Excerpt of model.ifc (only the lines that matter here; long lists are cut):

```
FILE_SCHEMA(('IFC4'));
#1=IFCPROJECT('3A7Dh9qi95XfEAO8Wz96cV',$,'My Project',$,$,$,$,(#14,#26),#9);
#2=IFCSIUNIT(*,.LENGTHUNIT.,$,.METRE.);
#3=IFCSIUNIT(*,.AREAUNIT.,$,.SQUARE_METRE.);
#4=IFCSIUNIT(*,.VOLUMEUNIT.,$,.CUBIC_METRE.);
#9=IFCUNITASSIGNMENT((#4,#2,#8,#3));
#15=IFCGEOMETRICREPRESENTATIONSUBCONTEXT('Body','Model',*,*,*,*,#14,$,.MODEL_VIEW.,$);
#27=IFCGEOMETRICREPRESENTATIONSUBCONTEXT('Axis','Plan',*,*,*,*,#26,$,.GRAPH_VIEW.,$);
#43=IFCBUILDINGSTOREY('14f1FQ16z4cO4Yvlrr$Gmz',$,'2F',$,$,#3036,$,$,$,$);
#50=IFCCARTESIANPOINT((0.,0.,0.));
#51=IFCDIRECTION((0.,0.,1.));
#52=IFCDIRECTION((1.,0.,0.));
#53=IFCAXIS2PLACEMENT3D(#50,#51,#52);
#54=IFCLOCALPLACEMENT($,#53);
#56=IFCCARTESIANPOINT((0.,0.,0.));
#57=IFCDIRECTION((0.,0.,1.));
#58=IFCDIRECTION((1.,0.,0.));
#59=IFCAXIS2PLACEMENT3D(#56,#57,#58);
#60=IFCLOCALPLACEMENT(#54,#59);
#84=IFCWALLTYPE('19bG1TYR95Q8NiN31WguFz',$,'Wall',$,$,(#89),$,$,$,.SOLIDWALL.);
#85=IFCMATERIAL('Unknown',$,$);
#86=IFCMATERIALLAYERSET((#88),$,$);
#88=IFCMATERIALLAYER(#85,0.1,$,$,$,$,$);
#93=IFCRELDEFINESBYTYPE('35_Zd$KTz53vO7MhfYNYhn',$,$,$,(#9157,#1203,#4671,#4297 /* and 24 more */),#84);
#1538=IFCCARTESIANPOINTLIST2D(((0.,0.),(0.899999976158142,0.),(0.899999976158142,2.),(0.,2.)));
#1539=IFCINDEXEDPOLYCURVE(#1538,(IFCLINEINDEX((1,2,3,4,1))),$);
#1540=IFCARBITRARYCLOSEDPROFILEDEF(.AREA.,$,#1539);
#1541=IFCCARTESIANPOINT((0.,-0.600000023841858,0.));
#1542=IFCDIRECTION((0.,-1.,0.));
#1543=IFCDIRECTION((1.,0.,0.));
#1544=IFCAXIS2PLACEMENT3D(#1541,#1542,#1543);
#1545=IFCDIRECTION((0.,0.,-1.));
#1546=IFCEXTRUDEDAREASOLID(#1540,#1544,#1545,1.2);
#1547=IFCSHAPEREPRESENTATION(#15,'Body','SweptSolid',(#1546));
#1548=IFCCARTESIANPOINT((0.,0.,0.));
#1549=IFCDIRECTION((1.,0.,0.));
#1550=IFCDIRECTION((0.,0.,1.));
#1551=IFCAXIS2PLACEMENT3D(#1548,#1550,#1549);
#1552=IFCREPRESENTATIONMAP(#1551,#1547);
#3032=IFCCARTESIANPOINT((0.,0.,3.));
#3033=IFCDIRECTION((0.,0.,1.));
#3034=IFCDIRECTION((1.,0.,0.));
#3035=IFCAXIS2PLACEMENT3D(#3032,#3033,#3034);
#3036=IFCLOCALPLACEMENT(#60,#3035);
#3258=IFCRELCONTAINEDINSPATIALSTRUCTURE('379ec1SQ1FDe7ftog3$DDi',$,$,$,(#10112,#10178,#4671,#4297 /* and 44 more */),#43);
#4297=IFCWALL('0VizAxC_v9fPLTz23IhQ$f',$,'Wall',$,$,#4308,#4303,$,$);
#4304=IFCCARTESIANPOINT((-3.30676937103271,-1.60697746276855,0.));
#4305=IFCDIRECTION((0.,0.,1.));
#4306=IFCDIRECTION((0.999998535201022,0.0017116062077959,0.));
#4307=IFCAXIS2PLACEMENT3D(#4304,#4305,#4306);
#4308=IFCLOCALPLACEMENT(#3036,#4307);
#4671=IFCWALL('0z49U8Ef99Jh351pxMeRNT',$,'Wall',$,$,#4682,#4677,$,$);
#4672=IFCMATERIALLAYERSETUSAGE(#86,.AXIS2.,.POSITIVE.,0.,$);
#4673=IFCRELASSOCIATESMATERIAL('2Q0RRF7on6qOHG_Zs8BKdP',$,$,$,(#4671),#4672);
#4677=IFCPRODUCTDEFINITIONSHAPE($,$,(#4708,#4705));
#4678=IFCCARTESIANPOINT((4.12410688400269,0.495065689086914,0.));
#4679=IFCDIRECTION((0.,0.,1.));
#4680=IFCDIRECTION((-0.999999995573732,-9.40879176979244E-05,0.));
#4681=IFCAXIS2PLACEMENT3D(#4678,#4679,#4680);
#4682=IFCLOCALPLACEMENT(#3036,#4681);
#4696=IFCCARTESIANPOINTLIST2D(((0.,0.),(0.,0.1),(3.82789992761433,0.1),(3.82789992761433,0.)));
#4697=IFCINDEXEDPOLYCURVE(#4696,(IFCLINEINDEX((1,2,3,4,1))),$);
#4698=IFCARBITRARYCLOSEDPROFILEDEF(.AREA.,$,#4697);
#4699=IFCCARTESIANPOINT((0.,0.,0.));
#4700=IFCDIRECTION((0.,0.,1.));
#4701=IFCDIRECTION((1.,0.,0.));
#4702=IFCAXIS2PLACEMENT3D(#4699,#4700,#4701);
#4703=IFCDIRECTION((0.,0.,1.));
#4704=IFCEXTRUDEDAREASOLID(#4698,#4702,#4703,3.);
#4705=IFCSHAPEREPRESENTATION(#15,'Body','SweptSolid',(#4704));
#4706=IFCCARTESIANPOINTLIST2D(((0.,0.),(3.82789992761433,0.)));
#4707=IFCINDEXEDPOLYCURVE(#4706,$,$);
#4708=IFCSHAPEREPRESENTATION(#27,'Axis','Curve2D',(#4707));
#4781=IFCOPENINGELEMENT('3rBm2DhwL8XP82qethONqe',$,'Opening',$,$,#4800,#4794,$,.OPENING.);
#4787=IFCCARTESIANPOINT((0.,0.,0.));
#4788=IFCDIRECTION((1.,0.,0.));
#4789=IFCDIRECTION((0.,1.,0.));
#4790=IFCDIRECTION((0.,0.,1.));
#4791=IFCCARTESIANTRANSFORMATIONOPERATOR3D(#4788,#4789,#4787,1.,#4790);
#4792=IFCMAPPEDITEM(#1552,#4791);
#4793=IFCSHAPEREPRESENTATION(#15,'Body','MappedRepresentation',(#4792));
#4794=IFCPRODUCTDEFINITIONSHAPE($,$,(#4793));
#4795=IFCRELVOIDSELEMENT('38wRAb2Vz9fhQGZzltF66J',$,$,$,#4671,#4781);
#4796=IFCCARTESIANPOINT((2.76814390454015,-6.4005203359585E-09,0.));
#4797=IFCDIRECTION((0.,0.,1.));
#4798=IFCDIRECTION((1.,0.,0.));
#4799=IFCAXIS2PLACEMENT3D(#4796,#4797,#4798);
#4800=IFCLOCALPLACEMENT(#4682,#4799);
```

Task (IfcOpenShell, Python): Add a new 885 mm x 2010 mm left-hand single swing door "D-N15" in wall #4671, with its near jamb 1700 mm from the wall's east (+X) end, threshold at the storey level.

```python
import numpy as np
import ifcopenshell
import ifcopenshell.api.feature
import ifcopenshell.api.geometry
import ifcopenshell.api.root
import ifcopenshell.api.spatial
import ifcopenshell.geom
import ifcopenshell.util.element
import ifcopenshell.util.placement
import ifcopenshell.util.representation
import ifcopenshell.util.shape
import ifcopenshell.util.unit

model = ifcopenshell.open("model.ifc")
unit_scale = ifcopenshell.util.unit.calculate_unit_scale(model)
settings = ifcopenshell.geom.settings()


def volume(element):
    """Net volume in cubic metres, openings subtracted."""
    shape = ifcopenshell.geom.create_shape(settings, element)
    return ifcopenshell.util.shape.get_volume(shape.geometry)


wall = model.by_id(4671)
storey = ifcopenshell.util.element.get_container(wall, ifc_class="IfcBuildingStorey")
context = ifcopenshell.util.representation.get_context(model, "Model", "Body", "MODEL_VIEW")
before = volume(wall)

width, height, from_end, sill = 0.885, 2.01, 1.7, 0.0  # metres

# The wall runs along its own X axis, and the end named is its -X end.
wall_shape = ifcopenshell.geom.create_shape(settings, wall)
x, y, z = ifcopenshell.util.shape.get_vertices(wall_shape.geometry).T
start = x.min() + from_end
face, thickness = float(y.min()), float(y.max() - y.min())
wall_matrix = ifcopenshell.util.placement.get_local_placement(wall.ObjectPlacement)
level = ifcopenshell.util.placement.get_local_placement(storey.ObjectPlacement)[2, 3]


def in_wall(x, y):
    """Placement at x, y metres in the wall's axes, at sill height."""
    matrix = wall_matrix.copy()
    matrix[:, 3] = wall_matrix @ np.array([x / unit_scale, y / unit_scale, 0.0, 1.0])
    matrix[2, 3] = level + sill / unit_scale
    return matrix


# Opening: a box that overshoots both wall faces by 50 mm.
opening = ifcopenshell.api.root.create_entity(model, ifc_class="IfcOpeningElement", predefined_type="OPENING")
box = ifcopenshell.api.geometry.add_wall_representation(
    model, context=context, length=width, height=height, thickness=thickness + 0.1
)
ifcopenshell.api.geometry.assign_representation(model, product=opening, representation=box)
ifcopenshell.api.geometry.edit_object_placement(model, product=opening, matrix=in_wall(start, face - 0.05), is_si=False)
ifcopenshell.api.feature.add_feature(model, feature=opening, element=wall)

door = ifcopenshell.api.root.create_entity(model, ifc_class="IfcDoor", name="D-N15", predefined_type="DOOR")
door.OverallWidth, door.OverallHeight = width / unit_scale, height / unit_scale
door.OperationType = "SINGLE_SWING_LEFT"
body = ifcopenshell.api.geometry.add_door_representation(
    model,
    context=context,
    overall_width=door.OverallWidth,
    overall_height=door.OverallHeight,
    operation_type="SINGLE_SWING_LEFT",
    lining_properties={"LiningDepth": thickness / unit_scale, "ThresholdDepth": thickness / unit_scale},
)
ifcopenshell.api.geometry.assign_representation(model, product=door, representation=body)
ifcopenshell.api.spatial.assign_container(model, products=[door], relating_structure=storey)
ifcopenshell.api.feature.add_filling(model, opening=opening, element=door)

# The lining spans the wall, so the door starts at the wall face.
ifcopenshell.api.geometry.edit_object_placement(model, product=door, matrix=in_wall(start, face), is_si=False)

after = volume(wall)

print(f"wall volume {before:.3f} -> {after:.3f} m3")

model.write("model_v2.ifc")
```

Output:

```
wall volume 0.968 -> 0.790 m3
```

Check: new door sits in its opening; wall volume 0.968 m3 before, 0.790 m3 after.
